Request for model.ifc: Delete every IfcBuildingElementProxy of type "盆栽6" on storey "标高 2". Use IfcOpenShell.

First a look at what the model holds.

```python
import ifcopenshell
import ifcopenshell.util.element

model = ifcopenshell.open("model.ifc")
print(model.schema)
storey = next(s for s in model.by_type("IfcBuildingStorey") if s.Name == "标高 2")
proxies = [e for e in ifcopenshell.util.element.get_decomposition(storey) if e.is_a("IfcBuildingElementProxy")]
seen = {}
for e in proxies:
    element_type = ifcopenshell.util.element.get_type(e)
    name = element_type.Name if element_type not in (None, e) else None
    seen[name] = seen.get(name, 0) + 1
for name, count in sorted(seen.items(), key=str):
    print(count, "x", name)
```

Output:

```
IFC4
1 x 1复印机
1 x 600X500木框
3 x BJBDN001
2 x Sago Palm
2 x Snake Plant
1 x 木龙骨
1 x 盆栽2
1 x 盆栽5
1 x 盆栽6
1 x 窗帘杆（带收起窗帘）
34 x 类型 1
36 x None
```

```python
import ifcopenshell
import ifcopenshell.api.root
import ifcopenshell.util.element

model = ifcopenshell.open("model.ifc")

storey = next(s for s in model.by_type("IfcBuildingStorey") if s.Name == "标高 2")
proxies = [e for e in ifcopenshell.util.element.get_decomposition(storey) if e.is_a("IfcBuildingElementProxy")]
targets = [e for e in proxies if (t := ifcopenshell.util.element.get_type(e)) not in (None, e) and t.Name == "盆栽6"]

for e in targets:
    ifcopenshell.api.root.remove_product(model, product=e)
print(len(targets), "removed")

model.write("model_rev.ifc")
```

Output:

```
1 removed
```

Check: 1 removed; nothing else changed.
